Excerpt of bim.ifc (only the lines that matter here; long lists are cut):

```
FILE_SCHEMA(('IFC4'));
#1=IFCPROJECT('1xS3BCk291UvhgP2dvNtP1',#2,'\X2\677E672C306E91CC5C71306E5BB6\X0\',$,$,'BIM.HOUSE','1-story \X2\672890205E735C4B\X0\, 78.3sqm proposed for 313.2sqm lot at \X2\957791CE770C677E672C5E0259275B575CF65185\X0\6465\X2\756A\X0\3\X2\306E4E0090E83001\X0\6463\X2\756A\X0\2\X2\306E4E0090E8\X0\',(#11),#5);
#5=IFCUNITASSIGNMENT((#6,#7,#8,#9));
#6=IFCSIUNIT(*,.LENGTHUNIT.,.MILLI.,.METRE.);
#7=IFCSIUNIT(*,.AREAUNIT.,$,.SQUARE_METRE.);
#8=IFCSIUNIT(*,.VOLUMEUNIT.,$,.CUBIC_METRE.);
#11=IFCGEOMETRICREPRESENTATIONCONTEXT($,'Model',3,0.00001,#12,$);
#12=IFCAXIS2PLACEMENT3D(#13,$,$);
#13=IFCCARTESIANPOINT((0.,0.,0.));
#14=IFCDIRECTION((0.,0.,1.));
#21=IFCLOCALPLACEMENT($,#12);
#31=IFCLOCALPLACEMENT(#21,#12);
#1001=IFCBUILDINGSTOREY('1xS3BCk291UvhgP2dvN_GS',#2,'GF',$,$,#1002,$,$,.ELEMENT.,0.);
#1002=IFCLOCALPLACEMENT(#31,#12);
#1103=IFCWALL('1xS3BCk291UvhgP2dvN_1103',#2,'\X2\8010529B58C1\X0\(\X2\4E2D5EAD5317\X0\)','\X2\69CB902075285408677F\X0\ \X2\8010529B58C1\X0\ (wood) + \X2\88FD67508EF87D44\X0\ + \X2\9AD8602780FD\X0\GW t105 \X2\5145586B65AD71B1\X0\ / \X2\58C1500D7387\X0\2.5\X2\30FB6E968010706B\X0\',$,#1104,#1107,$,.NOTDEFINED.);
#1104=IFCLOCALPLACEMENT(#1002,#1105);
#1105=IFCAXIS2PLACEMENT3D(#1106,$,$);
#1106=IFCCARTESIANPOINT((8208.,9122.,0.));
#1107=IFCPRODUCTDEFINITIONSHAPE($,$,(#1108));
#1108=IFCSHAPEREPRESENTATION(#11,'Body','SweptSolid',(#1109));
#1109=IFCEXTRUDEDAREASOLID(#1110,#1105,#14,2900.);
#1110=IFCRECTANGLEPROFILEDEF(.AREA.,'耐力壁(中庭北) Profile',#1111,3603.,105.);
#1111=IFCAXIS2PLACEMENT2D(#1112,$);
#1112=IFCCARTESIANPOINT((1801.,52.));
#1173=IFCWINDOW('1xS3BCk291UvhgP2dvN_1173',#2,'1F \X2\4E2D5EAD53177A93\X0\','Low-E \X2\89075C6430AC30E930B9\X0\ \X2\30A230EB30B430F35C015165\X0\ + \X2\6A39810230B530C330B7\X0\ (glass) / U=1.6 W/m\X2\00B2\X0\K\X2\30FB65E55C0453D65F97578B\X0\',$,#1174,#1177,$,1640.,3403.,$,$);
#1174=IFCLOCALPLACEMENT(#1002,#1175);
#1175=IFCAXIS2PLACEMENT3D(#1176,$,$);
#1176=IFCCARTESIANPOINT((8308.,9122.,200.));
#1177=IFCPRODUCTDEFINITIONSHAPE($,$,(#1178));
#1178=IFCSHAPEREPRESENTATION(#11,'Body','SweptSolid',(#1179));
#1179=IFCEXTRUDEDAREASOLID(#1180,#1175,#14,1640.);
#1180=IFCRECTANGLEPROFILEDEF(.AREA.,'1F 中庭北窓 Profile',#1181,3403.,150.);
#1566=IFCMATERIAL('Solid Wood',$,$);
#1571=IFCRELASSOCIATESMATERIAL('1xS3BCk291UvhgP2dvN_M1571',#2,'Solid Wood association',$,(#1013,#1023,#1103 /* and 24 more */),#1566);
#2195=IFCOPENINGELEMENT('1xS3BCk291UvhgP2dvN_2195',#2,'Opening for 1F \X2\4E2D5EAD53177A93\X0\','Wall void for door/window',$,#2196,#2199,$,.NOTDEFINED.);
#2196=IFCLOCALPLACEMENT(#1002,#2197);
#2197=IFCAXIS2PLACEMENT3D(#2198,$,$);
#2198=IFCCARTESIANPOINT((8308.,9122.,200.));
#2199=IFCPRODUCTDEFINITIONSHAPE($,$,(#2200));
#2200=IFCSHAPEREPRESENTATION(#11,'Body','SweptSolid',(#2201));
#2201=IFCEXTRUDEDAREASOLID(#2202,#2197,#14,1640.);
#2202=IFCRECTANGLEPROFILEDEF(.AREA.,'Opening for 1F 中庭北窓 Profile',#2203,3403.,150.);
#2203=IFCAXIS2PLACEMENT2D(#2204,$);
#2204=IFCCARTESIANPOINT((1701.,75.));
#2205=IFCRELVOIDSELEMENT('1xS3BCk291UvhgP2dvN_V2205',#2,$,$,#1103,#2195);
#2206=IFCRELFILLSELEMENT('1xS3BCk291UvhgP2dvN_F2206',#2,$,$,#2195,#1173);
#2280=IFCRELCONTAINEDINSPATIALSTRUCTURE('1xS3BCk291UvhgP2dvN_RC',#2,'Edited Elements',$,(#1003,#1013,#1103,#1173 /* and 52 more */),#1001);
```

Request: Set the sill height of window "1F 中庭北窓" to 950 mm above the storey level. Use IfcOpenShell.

```python
import numpy as np
import ifcopenshell
import ifcopenshell.api.geometry
import ifcopenshell.geom
import ifcopenshell.util.element
import ifcopenshell.util.placement
import ifcopenshell.util.shape
import ifcopenshell.util.unit

model = ifcopenshell.open("bim.ifc")
unit_scale = ifcopenshell.util.unit.calculate_unit_scale(model)

window = model.by_guid("1xS3BCk291UvhgP2dvN_1173")
opening = window.FillsVoids[0].RelatingOpeningElement
storey = ifcopenshell.util.element.get_container(window, ifc_class="IfcBuildingStorey")
level = ifcopenshell.util.placement.get_local_placement(storey.ObjectPlacement)[2, 3]

# The opening's origin need not be at the sill, so measure its lowest point.
shape = ifcopenshell.geom.create_shape(ifcopenshell.geom.settings(), opening)
bottom = ifcopenshell.util.shape.get_shape_bottom_elevation(shape, shape.geometry) / unit_scale
dz = level + 950.0 - bottom

shift = np.array([0.0, 0.0, dz])
# The window is not placed relative to its opening, so move both.
for product in (opening, window):
    matrix = ifcopenshell.util.placement.get_local_placement(product.ObjectPlacement)
    matrix[:3, 3] += shift
    ifcopenshell.api.geometry.edit_object_placement(model, product=product, matrix=matrix, is_si=False)

print(f"moved by {dz * unit_scale:+.3f} m")

model.write("bim_edited.ifc")
```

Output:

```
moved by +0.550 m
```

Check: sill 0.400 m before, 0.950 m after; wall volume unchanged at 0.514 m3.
